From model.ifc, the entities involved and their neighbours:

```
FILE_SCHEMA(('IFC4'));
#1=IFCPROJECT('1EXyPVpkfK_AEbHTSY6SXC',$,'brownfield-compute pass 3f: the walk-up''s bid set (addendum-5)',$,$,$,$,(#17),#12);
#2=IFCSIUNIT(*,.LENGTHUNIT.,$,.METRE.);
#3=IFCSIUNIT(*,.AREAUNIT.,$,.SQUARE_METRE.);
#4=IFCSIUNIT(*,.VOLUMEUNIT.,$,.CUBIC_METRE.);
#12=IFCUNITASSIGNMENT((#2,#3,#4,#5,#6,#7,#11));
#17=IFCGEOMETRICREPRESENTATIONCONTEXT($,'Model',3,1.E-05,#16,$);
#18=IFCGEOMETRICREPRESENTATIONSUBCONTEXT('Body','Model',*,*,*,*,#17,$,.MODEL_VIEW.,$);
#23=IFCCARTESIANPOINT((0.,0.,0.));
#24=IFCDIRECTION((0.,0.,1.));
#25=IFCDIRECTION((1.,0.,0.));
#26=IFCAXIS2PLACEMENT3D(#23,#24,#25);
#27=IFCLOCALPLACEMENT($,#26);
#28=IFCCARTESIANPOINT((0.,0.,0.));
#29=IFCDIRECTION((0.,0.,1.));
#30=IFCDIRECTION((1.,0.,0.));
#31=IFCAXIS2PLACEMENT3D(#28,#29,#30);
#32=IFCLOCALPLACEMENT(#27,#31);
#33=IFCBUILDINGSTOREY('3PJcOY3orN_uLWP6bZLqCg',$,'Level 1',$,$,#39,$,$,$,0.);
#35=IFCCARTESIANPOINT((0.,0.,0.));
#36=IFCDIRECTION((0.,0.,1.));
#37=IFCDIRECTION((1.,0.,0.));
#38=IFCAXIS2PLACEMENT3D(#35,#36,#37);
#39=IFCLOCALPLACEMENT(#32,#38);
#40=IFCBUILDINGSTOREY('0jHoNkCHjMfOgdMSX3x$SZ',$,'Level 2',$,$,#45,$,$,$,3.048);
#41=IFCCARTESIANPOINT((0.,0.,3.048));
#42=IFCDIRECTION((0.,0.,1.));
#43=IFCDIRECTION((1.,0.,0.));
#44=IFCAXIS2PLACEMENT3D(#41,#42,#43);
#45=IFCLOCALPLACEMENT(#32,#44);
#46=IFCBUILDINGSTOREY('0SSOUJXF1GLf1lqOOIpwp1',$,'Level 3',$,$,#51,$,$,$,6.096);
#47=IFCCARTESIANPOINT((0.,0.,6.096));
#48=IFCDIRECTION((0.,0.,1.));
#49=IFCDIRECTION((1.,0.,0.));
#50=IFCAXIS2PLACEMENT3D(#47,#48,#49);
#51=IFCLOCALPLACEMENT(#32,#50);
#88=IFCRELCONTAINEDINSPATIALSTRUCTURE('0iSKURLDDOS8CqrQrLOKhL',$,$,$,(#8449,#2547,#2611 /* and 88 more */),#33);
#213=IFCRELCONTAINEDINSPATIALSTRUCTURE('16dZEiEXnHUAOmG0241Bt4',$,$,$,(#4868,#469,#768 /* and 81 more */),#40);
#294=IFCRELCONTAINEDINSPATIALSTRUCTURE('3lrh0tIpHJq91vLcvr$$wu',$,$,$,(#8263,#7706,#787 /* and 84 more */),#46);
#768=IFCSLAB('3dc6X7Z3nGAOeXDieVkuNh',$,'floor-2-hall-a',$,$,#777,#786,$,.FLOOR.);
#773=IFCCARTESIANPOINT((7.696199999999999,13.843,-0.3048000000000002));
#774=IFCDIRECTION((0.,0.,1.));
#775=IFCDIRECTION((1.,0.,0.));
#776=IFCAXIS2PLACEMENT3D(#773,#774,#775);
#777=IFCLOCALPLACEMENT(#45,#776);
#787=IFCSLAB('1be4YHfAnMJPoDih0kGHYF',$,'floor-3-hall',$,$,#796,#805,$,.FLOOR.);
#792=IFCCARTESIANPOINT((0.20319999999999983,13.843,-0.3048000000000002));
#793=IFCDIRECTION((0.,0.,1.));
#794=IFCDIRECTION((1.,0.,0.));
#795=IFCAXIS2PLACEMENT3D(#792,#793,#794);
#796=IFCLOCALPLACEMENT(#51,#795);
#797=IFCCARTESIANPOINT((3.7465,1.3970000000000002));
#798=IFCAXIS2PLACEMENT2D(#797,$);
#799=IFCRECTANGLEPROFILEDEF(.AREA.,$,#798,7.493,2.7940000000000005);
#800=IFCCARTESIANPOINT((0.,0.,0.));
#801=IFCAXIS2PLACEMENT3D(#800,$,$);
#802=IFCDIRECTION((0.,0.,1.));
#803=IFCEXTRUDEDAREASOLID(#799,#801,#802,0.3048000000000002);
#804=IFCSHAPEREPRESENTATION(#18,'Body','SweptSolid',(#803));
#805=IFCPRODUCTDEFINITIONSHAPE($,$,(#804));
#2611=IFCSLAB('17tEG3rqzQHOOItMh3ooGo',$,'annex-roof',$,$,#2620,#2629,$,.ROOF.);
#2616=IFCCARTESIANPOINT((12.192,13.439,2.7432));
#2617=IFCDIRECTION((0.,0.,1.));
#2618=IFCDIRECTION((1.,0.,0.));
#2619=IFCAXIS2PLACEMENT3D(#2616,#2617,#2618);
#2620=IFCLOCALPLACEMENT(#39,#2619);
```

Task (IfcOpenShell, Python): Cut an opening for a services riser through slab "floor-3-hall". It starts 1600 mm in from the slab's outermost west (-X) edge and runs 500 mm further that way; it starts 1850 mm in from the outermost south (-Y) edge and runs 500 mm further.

```python
import numpy as np
import ifcopenshell
import ifcopenshell.api.feature
import ifcopenshell.api.geometry
import ifcopenshell.api.root
import ifcopenshell.geom
import ifcopenshell.util.placement
import ifcopenshell.util.representation
import ifcopenshell.util.shape
import ifcopenshell.util.unit

model = ifcopenshell.open("model.ifc")
unit_scale = ifcopenshell.util.unit.calculate_unit_scale(model)
settings = ifcopenshell.geom.settings()


def volume(element):
    """Net volume in cubic metres, openings subtracted."""
    shape = ifcopenshell.geom.create_shape(settings, element)
    return ifcopenshell.util.shape.get_volume(shape.geometry)


slab = model.by_guid("1be4YHfAnMJPoDih0kGHYF")
before = volume(slab)

# Extent in the slab's own axes, in metres. The edges named are its -X and -Y sides.
slab_shape = ifcopenshell.geom.create_shape(settings, slab)
vertices = ifcopenshell.util.shape.get_vertices(slab_shape.geometry)
x_min, y_min, bottom = vertices.min(axis=0)
top = vertices[:, 2].max()

opening = ifcopenshell.api.root.create_entity(model, ifc_class="IfcOpeningElement", name="Services riser opening", predefined_type="OPENING")
context = ifcopenshell.util.representation.get_context(model, "Model", "Body", "MODEL_VIEW")
width, depth = 0.5, 0.5
outline = [(0.0, 0.0), (width, 0.0), (width, depth), (0.0, depth), (0.0, 0.0)]
# Overshoot both faces by 50 mm so the cut is clean.
shape = ifcopenshell.api.geometry.add_slab_representation(
    model, context=context, depth=top - bottom + 0.1, polyline=outline
)
ifcopenshell.api.geometry.assign_representation(model, product=opening, representation=shape)

matrix = ifcopenshell.util.placement.get_local_placement(slab.ObjectPlacement)
matrix[:, 3] = matrix @ np.append(np.array([x_min + 1.6, y_min + 1.85, bottom - 0.05]) / unit_scale, 1.0)
ifcopenshell.api.geometry.edit_object_placement(model, product=opening, matrix=matrix, is_si=False)
ifcopenshell.api.feature.add_feature(model, feature=opening, element=slab)

after = volume(slab)

print(f"slab volume {before:.3f} -> {after:.3f} m3")

model.write("model_rev.ifc")
```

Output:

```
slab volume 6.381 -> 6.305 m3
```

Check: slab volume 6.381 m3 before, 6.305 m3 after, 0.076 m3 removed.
